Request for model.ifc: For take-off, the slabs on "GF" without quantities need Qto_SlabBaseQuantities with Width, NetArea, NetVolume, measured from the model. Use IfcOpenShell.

First a look at what the model holds.

```python
import ifcopenshell
import ifcopenshell.util.element
import ifcopenshell.util.unit

model = ifcopenshell.open("model.ifc")
print(model.schema)
for unit_type in ("LENGTHUNIT", "AREAUNIT", "VOLUMEUNIT"):
    print(unit_type, ifcopenshell.util.unit.calculate_unit_scale(model, unit_type))
storey = next(s for s in model.by_type("IfcBuildingStorey") if s.Name == "GF")
slabs = [e for e in ifcopenshell.util.element.get_decomposition(storey) if e.is_a("IfcSlab")]
for e in sorted(slabs, key=lambda e: e.id()):
    print(e.id(), e.is_a(), e.Name, list(ifcopenshell.util.element.get_psets(e, qtos_only=True)), sep=" | ")
```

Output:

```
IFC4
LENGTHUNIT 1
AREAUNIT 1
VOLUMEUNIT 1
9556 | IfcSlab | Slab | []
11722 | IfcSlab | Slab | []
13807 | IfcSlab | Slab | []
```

```python
import ifcopenshell
import ifcopenshell.api.pset
import ifcopenshell.geom
import ifcopenshell.util.element
import ifcopenshell.util.shape
import ifcopenshell.util.unit

model = ifcopenshell.open("model.ifc")
unit_scale = ifcopenshell.util.unit.calculate_unit_scale(model)
area_scale = ifcopenshell.util.unit.calculate_unit_scale(model, "AREAUNIT")
volume_scale = ifcopenshell.util.unit.calculate_unit_scale(model, "VOLUMEUNIT")
settings = ifcopenshell.geom.settings()

storey = next(s for s in model.by_type("IfcBuildingStorey") if s.Name == "GF")
slabs = [e for e in ifcopenshell.util.element.get_decomposition(storey) if e.is_a("IfcSlab")]

for e in sorted(slabs, key=lambda e: e.id()):
    if ifcopenshell.util.element.get_psets(e, qtos_only=True, should_inherit=False):
        continue
    # Geometry comes back in metres, in the element's own axes.
    shape = ifcopenshell.geom.create_shape(settings, e)
    values = {
        "Width": ifcopenshell.util.shape.get_z(shape.geometry) / unit_scale,
        "NetArea": ifcopenshell.util.shape.get_footprint_area(shape.geometry) / area_scale,
        "NetVolume": ifcopenshell.util.shape.get_volume(shape.geometry) / volume_scale,
    }
    qto = ifcopenshell.api.pset.add_qto(model, product=e, name="Qto_SlabBaseQuantities")
    ifcopenshell.api.pset.edit_qto(model, qto=qto, properties=values)
    print(e.id(), {k: round(v, 3) for k, v in values.items()})

model.write("model-out.ifc")
```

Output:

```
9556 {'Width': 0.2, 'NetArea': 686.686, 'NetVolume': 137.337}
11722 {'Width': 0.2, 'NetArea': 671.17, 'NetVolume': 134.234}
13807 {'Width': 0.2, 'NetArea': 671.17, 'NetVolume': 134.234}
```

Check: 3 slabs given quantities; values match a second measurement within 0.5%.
